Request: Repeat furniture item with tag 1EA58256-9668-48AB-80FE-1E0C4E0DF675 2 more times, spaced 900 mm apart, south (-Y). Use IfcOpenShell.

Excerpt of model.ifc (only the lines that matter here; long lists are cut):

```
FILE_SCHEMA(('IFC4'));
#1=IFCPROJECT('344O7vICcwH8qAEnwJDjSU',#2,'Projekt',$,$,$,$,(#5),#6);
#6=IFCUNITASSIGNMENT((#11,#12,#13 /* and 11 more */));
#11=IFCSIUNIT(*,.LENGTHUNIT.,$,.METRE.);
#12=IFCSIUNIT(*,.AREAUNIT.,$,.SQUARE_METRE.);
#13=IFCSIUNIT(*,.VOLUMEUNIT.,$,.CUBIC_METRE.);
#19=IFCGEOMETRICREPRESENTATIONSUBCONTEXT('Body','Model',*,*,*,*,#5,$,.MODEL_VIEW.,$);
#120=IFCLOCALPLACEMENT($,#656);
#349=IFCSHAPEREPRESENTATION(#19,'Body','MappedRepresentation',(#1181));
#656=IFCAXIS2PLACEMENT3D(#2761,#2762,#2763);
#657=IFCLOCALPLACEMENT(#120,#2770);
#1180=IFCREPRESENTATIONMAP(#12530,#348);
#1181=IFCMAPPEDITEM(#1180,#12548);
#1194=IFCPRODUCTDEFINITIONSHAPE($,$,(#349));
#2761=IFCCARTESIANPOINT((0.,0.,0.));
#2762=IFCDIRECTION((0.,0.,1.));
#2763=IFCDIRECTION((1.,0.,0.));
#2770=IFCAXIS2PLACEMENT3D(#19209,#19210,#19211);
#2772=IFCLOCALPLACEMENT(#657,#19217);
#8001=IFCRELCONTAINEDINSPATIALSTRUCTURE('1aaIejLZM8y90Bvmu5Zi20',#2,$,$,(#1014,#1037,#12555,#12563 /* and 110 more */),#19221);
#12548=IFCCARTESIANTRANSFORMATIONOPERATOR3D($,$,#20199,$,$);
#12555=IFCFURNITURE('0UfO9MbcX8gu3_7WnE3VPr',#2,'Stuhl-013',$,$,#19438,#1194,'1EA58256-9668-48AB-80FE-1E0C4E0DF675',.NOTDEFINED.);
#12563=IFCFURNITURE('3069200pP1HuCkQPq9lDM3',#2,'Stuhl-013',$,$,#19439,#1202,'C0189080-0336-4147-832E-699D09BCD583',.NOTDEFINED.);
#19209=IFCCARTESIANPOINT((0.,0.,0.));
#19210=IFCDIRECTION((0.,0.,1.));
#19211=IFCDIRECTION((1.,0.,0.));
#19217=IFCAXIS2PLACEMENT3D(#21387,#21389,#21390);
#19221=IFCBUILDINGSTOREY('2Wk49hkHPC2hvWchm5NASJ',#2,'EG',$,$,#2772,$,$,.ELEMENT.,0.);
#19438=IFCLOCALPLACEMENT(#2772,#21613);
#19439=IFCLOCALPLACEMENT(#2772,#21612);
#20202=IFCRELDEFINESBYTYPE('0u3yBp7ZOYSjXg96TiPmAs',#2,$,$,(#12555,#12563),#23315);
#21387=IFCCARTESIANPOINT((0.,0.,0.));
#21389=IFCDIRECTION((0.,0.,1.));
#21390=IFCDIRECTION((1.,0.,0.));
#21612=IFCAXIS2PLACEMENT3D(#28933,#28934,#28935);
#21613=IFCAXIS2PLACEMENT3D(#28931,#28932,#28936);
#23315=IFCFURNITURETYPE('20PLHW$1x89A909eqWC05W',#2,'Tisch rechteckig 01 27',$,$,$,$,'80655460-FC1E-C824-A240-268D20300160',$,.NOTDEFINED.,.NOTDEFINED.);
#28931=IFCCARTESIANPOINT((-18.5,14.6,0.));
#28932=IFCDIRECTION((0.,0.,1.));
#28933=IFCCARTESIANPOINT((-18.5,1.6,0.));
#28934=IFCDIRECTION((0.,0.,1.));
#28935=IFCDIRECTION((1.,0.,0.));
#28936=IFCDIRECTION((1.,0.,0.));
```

```python
import numpy as np
import ifcopenshell
import ifcopenshell.api.geometry
import ifcopenshell.api.root
import ifcopenshell.util.element
import ifcopenshell.util.placement
import ifcopenshell.util.unit

model = ifcopenshell.open("model.ifc")
unit_scale = ifcopenshell.util.unit.calculate_unit_scale(model)


def reuse_history(source, copy):
    """copy_class also copies each property set's owner history, people and application; keep the originals."""
    for rel in copy.IsDefinedBy:
        if rel.is_a("IfcRelDefinesByProperties") and (history := rel.RelatingPropertyDefinition.OwnerHistory):
            rel.RelatingPropertyDefinition.OwnerHistory = source.OwnerHistory
            ifcopenshell.util.element.remove_deep2(model, history)


source = model.by_guid("0UfO9MbcX8gu3_7WnE3VPr")
base = ifcopenshell.util.placement.get_local_placement(source.ObjectPlacement)
step = np.array([0.0, -1.0, 0.0]) * 0.9 / unit_scale

for i in range(1, 3):
    copy = ifcopenshell.api.root.copy_class(model, product=source)
    copy.Representation = ifcopenshell.util.element.copy_deep(
        model, source.Representation, exclude=["IfcGeometricRepresentationContext", "IfcRepresentationMap"]
    )
    copy.Tag = None
    reuse_history(source, copy)
    matrix = base.copy()
    matrix[:3, 3] += i * step
    print("added at", matrix[:3, 3].round(3) + 0.0)
    ifcopenshell.api.geometry.edit_object_placement(model, product=copy, matrix=matrix, is_si=False)

model.write("model_edited.ifc")
```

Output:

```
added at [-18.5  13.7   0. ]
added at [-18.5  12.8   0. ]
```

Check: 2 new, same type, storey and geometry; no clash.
